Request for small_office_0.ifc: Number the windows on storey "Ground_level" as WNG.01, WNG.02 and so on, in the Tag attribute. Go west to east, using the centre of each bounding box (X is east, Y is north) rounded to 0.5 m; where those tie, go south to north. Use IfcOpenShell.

First a look at what the model holds.

```python
import ifcopenshell
import ifcopenshell.util.element
import ifcopenshell.util.placement

model = ifcopenshell.open("small_office_0.ifc")
print(model.schema)
storey = next(s for s in model.by_type("IfcBuildingStorey") if s.Name == "Ground_level")
windows = [e for e in ifcopenshell.util.element.get_decomposition(storey) if e.is_a("IfcWindow")]
for e in sorted(windows, key=lambda e: e.id()):
    origin = ifcopenshell.util.placement.get_local_placement(e.ObjectPlacement)[:3, 3]
    print(e.id(), e.Tag, e.Name, origin.round(2) + 0.0, sep=" | ")
```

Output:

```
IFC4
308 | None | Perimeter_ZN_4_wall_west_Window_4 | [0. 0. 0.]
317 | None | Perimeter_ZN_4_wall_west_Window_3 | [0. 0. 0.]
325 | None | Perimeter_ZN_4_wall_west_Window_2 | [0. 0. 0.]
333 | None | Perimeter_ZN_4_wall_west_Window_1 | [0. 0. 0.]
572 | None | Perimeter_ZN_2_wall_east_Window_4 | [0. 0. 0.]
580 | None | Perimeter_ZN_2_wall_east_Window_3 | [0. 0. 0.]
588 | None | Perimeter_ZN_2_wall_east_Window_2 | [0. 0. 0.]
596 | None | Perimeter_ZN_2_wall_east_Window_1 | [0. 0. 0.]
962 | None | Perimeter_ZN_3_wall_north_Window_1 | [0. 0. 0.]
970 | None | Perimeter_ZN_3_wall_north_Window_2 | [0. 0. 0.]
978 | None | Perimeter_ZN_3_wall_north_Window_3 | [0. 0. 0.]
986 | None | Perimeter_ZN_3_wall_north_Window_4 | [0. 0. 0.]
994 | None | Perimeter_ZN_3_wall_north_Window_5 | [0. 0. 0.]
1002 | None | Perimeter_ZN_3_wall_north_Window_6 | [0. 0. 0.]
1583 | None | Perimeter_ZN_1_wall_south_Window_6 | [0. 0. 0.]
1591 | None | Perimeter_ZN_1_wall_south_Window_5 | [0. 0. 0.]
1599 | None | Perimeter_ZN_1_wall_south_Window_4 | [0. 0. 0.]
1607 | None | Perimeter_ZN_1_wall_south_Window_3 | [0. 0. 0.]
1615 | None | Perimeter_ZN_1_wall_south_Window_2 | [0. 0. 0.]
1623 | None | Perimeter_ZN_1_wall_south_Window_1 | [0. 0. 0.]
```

```python
import ifcopenshell
import ifcopenshell.geom
import ifcopenshell.util.element
import ifcopenshell.util.shape

model = ifcopenshell.open("small_office_0.ifc")
settings = ifcopenshell.geom.settings()
settings.set("use-world-coords", True)


def centre(element):
    shape = ifcopenshell.geom.create_shape(settings, element)
    return ifcopenshell.util.shape.get_bbox_centroid(shape.geometry)


storey = next(s for s in model.by_type("IfcBuildingStorey") if s.Name == "Ground_level")
windows = [e for e in ifcopenshell.util.element.get_decomposition(storey) if e.is_a("IfcWindow")]

# Insertion points can sit at a corner or the storey origin, so sort by the geometry (in metres).
centres = {e: centre(e) for e in windows}
windows.sort(key=lambda e: (round(centres[e][0] / 0.5), centres[e][1]))

for i, e in enumerate(windows, start=1):
    number = f"WNG.{i:02d}"
    e.Tag = number
    print(e.id(), number)

model.write("small_office_0_rev.ifc")
```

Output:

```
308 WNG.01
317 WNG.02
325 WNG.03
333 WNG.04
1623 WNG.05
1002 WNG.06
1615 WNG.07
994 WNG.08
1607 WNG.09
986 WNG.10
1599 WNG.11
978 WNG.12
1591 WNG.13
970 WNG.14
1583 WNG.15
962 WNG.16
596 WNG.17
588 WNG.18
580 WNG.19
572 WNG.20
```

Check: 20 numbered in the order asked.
